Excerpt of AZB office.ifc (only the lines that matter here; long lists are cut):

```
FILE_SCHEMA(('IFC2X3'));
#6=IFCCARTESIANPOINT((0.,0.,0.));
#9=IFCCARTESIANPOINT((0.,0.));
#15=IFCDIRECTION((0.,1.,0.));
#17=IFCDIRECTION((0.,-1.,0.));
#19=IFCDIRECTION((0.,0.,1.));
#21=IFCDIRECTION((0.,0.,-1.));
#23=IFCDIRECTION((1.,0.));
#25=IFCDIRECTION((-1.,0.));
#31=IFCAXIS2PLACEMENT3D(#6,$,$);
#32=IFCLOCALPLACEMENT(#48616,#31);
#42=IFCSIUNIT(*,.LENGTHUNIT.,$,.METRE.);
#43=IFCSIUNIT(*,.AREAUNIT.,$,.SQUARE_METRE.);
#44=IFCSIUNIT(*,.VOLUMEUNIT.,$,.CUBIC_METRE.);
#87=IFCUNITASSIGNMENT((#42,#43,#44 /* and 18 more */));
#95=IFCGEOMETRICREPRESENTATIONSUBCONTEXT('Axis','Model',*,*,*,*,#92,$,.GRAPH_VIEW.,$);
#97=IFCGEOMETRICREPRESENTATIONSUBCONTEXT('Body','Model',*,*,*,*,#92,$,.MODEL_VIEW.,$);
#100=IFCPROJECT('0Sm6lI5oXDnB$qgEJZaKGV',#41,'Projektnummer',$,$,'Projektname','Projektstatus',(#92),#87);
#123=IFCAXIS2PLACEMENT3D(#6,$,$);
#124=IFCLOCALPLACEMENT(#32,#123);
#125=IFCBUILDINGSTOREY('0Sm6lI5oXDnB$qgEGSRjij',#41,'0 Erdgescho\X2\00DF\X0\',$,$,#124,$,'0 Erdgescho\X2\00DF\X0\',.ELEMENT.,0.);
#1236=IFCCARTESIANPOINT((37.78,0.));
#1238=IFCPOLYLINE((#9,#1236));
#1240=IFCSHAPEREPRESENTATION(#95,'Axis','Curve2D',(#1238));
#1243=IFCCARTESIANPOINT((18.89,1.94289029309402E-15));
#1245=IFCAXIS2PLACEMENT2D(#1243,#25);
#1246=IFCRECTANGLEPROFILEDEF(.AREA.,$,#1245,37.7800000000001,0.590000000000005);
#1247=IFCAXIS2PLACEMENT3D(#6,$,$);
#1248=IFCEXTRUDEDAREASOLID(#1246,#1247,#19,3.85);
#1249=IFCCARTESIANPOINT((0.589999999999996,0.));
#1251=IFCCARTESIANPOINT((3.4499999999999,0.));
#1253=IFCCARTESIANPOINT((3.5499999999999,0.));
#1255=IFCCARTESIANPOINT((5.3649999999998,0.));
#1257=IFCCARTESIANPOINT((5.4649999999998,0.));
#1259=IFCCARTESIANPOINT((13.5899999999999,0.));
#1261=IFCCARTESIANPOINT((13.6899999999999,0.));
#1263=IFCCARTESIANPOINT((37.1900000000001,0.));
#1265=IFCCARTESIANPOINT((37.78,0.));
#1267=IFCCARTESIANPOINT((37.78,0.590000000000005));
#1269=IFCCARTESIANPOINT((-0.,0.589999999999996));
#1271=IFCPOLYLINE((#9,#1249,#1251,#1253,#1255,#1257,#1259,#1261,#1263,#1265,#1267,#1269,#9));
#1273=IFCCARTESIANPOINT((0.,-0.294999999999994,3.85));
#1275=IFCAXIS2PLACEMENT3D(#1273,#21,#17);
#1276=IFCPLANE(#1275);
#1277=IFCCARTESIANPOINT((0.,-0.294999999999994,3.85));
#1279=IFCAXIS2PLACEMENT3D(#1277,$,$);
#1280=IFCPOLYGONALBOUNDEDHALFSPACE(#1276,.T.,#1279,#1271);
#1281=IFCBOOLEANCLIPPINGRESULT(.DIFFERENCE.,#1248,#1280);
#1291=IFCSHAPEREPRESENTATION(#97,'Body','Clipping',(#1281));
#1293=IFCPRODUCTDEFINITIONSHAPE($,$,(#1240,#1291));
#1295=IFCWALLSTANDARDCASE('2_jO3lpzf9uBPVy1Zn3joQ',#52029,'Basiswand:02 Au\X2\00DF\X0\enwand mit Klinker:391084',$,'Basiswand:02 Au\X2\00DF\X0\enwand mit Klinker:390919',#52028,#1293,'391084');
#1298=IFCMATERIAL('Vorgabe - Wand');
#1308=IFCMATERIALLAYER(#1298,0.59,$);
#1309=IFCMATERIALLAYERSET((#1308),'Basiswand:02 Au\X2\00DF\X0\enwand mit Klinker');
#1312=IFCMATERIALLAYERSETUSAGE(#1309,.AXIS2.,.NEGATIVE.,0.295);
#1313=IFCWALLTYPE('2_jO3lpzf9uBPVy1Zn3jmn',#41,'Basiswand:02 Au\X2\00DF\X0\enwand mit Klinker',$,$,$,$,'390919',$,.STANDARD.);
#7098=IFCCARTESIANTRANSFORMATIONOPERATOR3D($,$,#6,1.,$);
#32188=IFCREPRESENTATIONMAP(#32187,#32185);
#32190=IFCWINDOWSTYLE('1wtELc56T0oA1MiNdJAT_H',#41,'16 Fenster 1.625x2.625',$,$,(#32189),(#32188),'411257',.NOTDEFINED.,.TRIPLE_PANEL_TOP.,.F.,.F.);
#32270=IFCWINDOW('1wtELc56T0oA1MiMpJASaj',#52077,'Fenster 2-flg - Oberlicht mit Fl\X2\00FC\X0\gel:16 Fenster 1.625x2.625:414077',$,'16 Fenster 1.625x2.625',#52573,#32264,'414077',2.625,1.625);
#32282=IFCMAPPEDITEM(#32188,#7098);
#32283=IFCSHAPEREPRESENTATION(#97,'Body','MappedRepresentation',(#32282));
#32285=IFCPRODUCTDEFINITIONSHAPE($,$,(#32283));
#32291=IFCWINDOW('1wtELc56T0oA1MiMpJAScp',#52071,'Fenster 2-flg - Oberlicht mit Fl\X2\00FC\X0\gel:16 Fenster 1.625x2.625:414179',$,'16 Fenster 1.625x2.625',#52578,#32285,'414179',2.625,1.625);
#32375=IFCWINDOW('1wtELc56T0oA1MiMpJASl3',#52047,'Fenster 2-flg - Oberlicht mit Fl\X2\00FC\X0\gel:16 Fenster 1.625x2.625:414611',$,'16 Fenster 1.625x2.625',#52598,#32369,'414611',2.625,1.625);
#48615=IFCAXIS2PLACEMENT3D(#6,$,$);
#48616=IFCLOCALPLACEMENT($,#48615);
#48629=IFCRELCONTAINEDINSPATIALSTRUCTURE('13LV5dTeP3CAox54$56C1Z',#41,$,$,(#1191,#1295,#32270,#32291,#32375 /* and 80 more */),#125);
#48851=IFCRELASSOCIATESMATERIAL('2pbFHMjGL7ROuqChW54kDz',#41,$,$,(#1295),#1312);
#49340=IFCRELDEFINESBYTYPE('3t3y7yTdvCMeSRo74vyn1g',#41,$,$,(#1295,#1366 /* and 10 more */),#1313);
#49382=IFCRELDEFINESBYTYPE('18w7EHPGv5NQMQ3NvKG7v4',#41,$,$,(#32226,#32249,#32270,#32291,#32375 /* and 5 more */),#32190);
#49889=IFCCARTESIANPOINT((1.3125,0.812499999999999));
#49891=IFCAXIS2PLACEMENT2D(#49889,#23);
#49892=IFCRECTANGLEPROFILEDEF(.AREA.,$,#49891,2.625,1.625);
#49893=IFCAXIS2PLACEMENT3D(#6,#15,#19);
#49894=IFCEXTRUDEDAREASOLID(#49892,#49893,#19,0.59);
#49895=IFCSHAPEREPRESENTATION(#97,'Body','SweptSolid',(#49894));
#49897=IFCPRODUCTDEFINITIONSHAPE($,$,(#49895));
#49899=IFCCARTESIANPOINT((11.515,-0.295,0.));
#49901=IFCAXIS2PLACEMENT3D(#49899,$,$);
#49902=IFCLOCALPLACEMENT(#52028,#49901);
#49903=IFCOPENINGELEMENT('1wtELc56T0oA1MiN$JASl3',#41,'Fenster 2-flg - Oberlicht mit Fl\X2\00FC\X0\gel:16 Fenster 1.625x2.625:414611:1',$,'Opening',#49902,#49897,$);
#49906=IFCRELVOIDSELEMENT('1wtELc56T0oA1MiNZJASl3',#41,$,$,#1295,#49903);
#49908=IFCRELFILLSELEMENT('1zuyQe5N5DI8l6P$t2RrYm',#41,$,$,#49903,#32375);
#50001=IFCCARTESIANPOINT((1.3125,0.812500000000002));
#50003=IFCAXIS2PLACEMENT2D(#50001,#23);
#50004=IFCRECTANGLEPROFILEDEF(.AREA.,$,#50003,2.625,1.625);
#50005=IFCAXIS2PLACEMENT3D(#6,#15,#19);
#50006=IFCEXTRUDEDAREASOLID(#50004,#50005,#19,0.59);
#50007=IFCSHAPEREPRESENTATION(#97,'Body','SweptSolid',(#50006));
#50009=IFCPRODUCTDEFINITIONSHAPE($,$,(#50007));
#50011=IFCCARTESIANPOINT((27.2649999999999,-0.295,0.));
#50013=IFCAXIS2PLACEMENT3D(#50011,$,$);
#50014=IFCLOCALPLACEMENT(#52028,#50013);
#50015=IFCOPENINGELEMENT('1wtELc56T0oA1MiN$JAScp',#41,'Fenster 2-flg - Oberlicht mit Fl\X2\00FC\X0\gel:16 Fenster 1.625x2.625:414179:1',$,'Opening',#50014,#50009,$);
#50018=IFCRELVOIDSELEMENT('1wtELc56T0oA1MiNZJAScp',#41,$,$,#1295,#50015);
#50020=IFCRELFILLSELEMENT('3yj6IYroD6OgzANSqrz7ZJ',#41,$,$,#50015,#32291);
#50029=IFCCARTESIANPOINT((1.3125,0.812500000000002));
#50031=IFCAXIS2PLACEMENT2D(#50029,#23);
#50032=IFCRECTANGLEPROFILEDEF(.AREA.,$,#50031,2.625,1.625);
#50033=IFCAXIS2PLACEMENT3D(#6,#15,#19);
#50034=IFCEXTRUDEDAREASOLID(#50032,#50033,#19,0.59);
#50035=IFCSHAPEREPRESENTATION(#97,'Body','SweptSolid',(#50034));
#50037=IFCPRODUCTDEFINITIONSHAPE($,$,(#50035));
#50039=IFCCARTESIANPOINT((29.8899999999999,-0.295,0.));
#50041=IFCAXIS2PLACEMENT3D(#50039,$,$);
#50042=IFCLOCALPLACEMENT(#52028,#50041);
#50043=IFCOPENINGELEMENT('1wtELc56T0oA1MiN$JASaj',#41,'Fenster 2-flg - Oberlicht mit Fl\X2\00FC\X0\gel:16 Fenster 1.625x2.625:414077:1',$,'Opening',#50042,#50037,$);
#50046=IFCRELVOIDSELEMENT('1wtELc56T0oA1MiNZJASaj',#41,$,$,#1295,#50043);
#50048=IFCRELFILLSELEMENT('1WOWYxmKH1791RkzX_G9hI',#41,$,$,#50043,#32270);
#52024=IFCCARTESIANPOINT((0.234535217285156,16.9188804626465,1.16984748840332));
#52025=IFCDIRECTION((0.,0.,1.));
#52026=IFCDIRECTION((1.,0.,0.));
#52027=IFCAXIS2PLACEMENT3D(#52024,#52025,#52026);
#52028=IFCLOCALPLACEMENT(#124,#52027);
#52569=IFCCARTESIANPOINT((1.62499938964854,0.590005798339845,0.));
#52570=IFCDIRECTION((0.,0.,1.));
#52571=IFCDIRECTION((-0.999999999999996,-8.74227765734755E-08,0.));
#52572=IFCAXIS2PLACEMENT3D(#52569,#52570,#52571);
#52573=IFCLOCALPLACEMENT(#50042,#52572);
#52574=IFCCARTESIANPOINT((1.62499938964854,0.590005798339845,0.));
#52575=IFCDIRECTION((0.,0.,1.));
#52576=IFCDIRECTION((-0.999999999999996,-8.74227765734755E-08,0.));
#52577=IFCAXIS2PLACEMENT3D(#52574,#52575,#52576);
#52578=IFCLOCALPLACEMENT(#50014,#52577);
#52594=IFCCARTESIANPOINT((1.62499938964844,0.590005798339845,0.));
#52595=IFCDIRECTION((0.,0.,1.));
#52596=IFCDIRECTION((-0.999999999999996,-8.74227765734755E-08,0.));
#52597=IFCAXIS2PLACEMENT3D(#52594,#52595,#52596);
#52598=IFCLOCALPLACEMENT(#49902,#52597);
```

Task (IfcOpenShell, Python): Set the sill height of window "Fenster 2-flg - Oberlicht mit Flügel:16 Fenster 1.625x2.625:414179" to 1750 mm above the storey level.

```python
import numpy as np
import ifcopenshell
import ifcopenshell.api.geometry
import ifcopenshell.geom
import ifcopenshell.util.element
import ifcopenshell.util.placement
import ifcopenshell.util.shape
import ifcopenshell.util.unit

model = ifcopenshell.open("AZB office.ifc")
unit_scale = ifcopenshell.util.unit.calculate_unit_scale(model)

window = model.by_guid("1wtELc56T0oA1MiMpJAScp")
opening = window.FillsVoids[0].RelatingOpeningElement
storey = ifcopenshell.util.element.get_container(window, ifc_class="IfcBuildingStorey")
level = ifcopenshell.util.placement.get_local_placement(storey.ObjectPlacement)[2, 3]

# The opening's origin need not be at the sill, so measure its lowest point.
shape = ifcopenshell.geom.create_shape(ifcopenshell.geom.settings(), opening)
bottom = ifcopenshell.util.shape.get_shape_bottom_elevation(shape, shape.geometry) / unit_scale
dz = level + 1.75 / unit_scale - bottom

shift = np.array([0.0, 0.0, dz])
# The window is placed relative to its opening, so it follows when the opening moves.
matrix = ifcopenshell.util.placement.get_local_placement(opening.ObjectPlacement)
matrix[:3, 3] += shift
ifcopenshell.api.geometry.edit_object_placement(
    model, product=opening, matrix=matrix, is_si=False, should_transform_children=True
)

print(f"moved by {dz * unit_scale:+.3f} m")

model.write("AZB office_edited.ifc")
```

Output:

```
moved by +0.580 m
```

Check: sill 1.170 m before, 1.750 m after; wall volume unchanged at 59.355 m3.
